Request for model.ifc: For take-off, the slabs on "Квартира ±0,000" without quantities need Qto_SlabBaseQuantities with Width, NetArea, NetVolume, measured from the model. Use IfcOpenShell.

First a look at what the model holds.

```python
import ifcopenshell
import ifcopenshell.util.element
import ifcopenshell.util.unit

model = ifcopenshell.open("model.ifc")
print(model.schema)
for unit_type in ("LENGTHUNIT", "AREAUNIT", "VOLUMEUNIT"):
    print(unit_type, ifcopenshell.util.unit.calculate_unit_scale(model, unit_type))
storey = next(s for s in model.by_type("IfcBuildingStorey") if s.Name == "Квартира ±0,000")
slabs = [e for e in ifcopenshell.util.element.get_decomposition(storey) if e.is_a("IfcSlab")]
for e in sorted(slabs, key=lambda e: e.id()):
    print(e.id(), e.is_a(), e.Name, list(ifcopenshell.util.element.get_psets(e, qtos_only=True)), sep=" | ")
```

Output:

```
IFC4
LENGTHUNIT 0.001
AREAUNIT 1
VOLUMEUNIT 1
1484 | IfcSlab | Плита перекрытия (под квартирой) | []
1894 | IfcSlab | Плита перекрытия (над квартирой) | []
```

```python
import ifcopenshell
import ifcopenshell.api.pset
import ifcopenshell.geom
import ifcopenshell.util.element
import ifcopenshell.util.shape
import ifcopenshell.util.unit

model = ifcopenshell.open("model.ifc")
unit_scale = ifcopenshell.util.unit.calculate_unit_scale(model)
area_scale = ifcopenshell.util.unit.calculate_unit_scale(model, "AREAUNIT")
volume_scale = ifcopenshell.util.unit.calculate_unit_scale(model, "VOLUMEUNIT")
settings = ifcopenshell.geom.settings()

storey = next(s for s in model.by_type("IfcBuildingStorey") if s.Name == "Квартира ±0,000")
slabs = [e for e in ifcopenshell.util.element.get_decomposition(storey) if e.is_a("IfcSlab")]

for e in sorted(slabs, key=lambda e: e.id()):
    if ifcopenshell.util.element.get_psets(e, qtos_only=True, should_inherit=False):
        continue
    # Geometry comes back in metres, in the element's own axes.
    shape = ifcopenshell.geom.create_shape(settings, e)
    values = {
        "Width": ifcopenshell.util.shape.get_z(shape.geometry) / unit_scale,
        "NetArea": ifcopenshell.util.shape.get_footprint_area(shape.geometry) / area_scale,
        "NetVolume": ifcopenshell.util.shape.get_volume(shape.geometry) / volume_scale,
    }
    qto = ifcopenshell.api.pset.add_qto(model, product=e, name="Qto_SlabBaseQuantities")
    ifcopenshell.api.pset.edit_qto(model, qto=qto, properties=values)
    print(e.id(), {k: round(v, 3) for k, v in values.items()})

model.write("model_updated.ifc")
```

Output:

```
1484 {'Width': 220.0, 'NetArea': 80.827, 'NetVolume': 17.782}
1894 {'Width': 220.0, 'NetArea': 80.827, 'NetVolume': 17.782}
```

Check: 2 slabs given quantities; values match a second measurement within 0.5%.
